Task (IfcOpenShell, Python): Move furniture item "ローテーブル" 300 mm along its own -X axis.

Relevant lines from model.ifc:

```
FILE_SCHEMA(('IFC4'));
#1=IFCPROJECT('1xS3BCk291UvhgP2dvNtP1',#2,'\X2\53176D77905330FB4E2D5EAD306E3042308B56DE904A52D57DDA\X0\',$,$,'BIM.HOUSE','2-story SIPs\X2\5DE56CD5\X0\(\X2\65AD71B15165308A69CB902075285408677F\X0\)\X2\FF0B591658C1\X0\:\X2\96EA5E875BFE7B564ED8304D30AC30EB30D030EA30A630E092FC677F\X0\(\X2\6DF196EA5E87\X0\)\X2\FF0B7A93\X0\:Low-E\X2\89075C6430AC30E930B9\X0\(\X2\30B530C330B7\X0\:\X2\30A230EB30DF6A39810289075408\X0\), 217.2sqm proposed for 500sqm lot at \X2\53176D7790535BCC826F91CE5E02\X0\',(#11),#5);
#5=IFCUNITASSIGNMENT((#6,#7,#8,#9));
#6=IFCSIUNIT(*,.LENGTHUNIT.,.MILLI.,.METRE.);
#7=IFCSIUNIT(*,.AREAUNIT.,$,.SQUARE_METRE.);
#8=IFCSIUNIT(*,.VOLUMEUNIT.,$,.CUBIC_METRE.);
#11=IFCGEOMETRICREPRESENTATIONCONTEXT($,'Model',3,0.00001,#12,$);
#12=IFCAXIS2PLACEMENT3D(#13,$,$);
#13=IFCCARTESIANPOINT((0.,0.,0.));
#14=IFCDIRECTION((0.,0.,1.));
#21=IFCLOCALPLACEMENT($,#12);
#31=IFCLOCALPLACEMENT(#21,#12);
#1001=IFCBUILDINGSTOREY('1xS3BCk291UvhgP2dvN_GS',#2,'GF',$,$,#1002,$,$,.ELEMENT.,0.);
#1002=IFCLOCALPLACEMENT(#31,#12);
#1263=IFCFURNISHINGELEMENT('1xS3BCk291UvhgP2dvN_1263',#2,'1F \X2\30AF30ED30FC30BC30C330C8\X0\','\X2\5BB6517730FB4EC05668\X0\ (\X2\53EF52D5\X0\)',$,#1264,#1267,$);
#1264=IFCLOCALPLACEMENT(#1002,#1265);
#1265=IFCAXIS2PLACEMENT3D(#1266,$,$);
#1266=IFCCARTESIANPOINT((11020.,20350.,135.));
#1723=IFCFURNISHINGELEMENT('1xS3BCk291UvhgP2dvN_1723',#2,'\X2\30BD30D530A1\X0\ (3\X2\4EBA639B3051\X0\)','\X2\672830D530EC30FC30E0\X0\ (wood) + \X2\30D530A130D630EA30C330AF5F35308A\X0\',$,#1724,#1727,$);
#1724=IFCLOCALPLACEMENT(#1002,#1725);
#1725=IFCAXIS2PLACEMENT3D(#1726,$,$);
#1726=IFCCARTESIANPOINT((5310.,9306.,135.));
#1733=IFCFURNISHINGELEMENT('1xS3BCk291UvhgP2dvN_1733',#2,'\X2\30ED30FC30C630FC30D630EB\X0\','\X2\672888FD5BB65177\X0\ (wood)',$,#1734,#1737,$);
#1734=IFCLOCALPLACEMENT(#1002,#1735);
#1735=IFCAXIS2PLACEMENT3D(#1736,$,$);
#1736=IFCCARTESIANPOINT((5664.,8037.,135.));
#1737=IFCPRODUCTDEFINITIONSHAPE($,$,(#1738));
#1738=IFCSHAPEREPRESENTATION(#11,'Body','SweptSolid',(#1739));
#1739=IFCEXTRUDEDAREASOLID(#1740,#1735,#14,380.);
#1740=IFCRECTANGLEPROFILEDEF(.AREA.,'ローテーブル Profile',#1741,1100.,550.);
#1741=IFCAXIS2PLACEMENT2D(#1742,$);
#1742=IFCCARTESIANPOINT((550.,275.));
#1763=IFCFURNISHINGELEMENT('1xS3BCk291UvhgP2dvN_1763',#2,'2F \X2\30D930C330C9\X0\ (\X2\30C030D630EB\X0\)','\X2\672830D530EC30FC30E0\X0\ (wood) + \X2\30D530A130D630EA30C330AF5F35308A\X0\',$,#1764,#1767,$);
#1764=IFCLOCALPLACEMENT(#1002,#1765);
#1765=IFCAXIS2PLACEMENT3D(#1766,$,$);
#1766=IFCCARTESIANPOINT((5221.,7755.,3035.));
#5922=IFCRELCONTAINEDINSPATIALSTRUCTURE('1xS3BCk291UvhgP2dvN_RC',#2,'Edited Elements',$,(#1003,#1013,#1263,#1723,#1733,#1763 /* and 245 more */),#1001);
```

```python
import ifcopenshell
import ifcopenshell.api.geometry
import ifcopenshell.util.placement

model = ifcopenshell.open("model.ifc")

item = model.by_guid("1xS3BCk291UvhgP2dvN_1733")
matrix = ifcopenshell.util.placement.get_local_placement(item.ObjectPlacement)
matrix[:3, 3] -= matrix[:3, 0] * 300.0
ifcopenshell.api.geometry.edit_object_placement(model, product=item, matrix=matrix, is_si=False)

print(ifcopenshell.util.placement.get_local_placement(item.ObjectPlacement).round(3) + 0.0)

model.write("model_rev.ifc")
```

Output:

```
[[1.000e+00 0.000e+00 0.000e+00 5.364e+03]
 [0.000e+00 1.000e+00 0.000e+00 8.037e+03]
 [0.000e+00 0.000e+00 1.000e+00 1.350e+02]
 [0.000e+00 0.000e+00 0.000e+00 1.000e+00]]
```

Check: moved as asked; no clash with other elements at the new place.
